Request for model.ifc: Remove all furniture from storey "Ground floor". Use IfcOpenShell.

First a look at what the model holds.

```python
import ifcopenshell
import ifcopenshell.util.element

model = ifcopenshell.open("model.ifc")
print(model.schema)
storey = next(s for s in model.by_type("IfcBuildingStorey") if s.Name == "Ground floor")
furniture = [e for e in ifcopenshell.util.element.get_decomposition(storey) if e.is_a("IfcFurnishingElement")]
seen = {}
for e in furniture:
    element_type = ifcopenshell.util.element.get_type(e)
    name = element_type.Name if element_type not in (None, e) else None
    seen[name] = seen.get(name, 0) + 1
for name, count in sorted(seen.items(), key=str):
    print(count, "x", name)
```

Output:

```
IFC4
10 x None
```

```python
import ifcopenshell
import ifcopenshell.api.root
import ifcopenshell.util.element

model = ifcopenshell.open("model.ifc")

storey = next(s for s in model.by_type("IfcBuildingStorey") if s.Name == "Ground floor")
furniture = [e for e in ifcopenshell.util.element.get_decomposition(storey) if e.is_a("IfcFurnishingElement")]

for e in furniture:
    ifcopenshell.api.root.remove_product(model, product=e)
print(len(furniture), "removed")

model.write("model-out.ifc")
```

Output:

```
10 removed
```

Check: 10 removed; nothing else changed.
